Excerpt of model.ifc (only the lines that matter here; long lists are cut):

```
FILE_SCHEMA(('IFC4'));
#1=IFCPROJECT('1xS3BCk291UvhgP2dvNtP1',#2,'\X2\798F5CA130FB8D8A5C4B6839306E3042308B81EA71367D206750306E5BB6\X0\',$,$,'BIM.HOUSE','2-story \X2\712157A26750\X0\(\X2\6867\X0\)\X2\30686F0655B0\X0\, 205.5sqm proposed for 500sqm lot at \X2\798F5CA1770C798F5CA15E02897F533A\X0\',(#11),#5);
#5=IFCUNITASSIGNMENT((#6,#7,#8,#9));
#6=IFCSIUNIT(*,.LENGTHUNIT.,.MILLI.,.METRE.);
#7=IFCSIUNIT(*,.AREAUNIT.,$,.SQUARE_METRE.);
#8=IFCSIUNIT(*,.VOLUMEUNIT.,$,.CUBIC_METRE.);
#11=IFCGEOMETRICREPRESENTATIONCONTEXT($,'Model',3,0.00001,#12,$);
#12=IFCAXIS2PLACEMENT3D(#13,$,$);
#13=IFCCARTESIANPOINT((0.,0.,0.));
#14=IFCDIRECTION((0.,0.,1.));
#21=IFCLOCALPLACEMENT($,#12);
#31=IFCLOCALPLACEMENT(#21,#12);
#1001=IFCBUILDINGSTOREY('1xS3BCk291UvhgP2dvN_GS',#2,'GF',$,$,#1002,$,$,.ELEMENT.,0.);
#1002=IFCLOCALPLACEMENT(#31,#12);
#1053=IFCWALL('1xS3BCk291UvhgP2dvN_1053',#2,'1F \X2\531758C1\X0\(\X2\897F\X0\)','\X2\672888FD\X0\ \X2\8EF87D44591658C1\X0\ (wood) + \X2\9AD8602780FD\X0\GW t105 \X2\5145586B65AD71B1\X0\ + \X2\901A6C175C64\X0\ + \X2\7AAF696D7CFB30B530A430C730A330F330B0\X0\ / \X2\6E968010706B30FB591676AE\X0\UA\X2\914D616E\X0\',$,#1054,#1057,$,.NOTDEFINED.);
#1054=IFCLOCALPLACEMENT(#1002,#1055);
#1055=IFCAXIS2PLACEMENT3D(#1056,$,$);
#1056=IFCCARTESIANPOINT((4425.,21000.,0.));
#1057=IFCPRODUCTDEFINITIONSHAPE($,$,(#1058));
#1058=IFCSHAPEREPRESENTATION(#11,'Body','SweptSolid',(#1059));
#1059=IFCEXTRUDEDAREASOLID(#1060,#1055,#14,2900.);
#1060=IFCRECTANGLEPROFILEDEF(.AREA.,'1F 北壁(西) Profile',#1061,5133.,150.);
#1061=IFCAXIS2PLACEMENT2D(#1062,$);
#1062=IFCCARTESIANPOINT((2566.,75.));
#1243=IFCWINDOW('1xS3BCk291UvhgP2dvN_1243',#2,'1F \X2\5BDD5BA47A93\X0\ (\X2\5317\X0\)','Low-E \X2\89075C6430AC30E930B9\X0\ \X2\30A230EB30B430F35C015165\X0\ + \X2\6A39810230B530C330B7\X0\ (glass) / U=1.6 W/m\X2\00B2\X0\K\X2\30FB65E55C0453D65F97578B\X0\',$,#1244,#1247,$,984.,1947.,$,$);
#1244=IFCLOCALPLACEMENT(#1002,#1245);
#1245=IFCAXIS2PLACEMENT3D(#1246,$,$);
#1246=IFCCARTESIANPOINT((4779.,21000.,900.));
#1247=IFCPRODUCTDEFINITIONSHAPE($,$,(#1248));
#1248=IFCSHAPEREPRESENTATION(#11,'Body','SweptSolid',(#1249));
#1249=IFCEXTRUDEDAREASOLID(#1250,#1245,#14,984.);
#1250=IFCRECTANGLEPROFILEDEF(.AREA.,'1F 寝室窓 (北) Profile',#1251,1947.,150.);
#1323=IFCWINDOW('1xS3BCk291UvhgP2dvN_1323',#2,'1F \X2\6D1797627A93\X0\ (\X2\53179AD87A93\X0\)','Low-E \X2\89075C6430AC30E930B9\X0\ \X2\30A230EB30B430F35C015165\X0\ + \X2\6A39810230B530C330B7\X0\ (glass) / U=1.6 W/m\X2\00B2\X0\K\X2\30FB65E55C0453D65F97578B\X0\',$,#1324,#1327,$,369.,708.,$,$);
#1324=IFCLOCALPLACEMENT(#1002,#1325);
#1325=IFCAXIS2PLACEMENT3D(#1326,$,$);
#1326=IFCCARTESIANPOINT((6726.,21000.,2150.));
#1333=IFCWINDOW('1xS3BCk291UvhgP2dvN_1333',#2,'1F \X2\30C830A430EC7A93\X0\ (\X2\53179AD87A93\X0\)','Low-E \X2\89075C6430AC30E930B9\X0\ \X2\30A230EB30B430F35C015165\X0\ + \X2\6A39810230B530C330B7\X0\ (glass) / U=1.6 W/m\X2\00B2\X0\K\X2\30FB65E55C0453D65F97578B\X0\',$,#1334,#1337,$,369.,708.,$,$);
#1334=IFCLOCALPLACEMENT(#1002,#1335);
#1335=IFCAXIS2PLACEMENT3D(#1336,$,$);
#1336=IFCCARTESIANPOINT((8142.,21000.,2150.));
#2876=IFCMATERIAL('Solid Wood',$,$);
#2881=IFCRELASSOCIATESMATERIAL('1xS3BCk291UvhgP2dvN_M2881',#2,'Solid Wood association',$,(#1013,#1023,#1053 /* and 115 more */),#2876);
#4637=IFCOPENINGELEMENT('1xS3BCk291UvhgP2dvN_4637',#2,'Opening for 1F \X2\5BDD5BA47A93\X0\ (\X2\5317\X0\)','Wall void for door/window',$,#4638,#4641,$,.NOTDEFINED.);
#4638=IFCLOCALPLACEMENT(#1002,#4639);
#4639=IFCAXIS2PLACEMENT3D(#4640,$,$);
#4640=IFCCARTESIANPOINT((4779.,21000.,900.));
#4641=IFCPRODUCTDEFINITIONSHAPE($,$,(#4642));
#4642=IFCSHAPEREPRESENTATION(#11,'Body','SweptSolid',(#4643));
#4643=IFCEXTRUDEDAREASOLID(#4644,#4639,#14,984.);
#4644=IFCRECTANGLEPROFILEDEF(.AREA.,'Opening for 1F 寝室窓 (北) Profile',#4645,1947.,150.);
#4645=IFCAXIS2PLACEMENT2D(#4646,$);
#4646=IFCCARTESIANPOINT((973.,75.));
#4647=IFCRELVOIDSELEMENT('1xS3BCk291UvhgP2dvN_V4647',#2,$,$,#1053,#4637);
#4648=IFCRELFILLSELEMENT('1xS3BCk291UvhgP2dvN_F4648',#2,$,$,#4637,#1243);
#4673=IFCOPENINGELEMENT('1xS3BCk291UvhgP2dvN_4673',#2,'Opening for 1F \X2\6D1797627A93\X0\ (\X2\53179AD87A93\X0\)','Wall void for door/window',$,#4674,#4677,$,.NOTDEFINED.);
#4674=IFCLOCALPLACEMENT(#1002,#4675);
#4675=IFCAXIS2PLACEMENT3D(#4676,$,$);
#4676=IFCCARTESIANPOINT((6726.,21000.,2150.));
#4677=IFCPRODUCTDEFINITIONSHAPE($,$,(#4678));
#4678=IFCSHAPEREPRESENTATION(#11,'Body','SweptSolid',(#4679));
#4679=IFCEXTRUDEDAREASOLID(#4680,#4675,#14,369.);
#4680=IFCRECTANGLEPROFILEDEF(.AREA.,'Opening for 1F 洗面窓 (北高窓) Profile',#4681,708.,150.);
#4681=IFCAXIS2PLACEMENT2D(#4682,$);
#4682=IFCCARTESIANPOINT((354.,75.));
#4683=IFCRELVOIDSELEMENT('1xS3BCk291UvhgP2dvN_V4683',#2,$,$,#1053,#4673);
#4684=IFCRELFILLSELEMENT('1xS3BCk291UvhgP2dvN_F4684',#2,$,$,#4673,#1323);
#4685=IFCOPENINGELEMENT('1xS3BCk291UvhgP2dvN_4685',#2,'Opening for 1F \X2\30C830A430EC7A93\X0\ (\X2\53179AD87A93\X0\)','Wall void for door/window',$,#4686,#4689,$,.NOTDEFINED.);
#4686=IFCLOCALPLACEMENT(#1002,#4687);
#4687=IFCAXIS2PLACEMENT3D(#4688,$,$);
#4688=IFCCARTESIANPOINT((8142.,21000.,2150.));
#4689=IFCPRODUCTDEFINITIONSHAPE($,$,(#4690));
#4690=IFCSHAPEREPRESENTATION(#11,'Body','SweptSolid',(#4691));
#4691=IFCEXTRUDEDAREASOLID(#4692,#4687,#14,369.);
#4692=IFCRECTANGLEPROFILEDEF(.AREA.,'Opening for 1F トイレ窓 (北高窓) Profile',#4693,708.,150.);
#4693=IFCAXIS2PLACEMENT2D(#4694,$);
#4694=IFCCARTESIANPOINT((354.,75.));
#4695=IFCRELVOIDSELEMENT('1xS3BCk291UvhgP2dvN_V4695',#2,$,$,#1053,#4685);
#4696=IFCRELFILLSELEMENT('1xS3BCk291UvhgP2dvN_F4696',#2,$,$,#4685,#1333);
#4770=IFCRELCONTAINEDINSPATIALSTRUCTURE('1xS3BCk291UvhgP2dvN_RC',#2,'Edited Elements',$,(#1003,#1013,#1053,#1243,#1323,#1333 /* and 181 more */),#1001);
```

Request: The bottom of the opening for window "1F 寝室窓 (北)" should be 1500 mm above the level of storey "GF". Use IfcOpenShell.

```python
import numpy as np
import ifcopenshell
import ifcopenshell.api.geometry
import ifcopenshell.geom
import ifcopenshell.util.element
import ifcopenshell.util.placement
import ifcopenshell.util.shape
import ifcopenshell.util.unit

model = ifcopenshell.open("model.ifc")
unit_scale = ifcopenshell.util.unit.calculate_unit_scale(model)

window = model.by_guid("1xS3BCk291UvhgP2dvN_1243")
opening = window.FillsVoids[0].RelatingOpeningElement
storey = ifcopenshell.util.element.get_container(window, ifc_class="IfcBuildingStorey")
level = ifcopenshell.util.placement.get_local_placement(storey.ObjectPlacement)[2, 3]

# The opening's origin need not be at the sill, so measure its lowest point.
shape = ifcopenshell.geom.create_shape(ifcopenshell.geom.settings(), opening)
bottom = ifcopenshell.util.shape.get_shape_bottom_elevation(shape, shape.geometry) / unit_scale
dz = level + 1500.0 - bottom

shift = np.array([0.0, 0.0, dz])
# The window is not placed relative to its opening, so move both.
for product in (opening, window):
    matrix = ifcopenshell.util.placement.get_local_placement(product.ObjectPlacement)
    matrix[:3, 3] += shift
    ifcopenshell.api.geometry.edit_object_placement(model, product=product, matrix=matrix, is_si=False)

print(f"moved by {dz * unit_scale:+.3f} m")

model.write("model_edited.ifc")
```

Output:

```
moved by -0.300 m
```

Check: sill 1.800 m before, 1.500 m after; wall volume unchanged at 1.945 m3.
